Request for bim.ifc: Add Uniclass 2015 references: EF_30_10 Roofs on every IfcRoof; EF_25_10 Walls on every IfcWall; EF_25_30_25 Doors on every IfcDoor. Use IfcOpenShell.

First a look at what the model holds.

```python
import ifcopenshell

model = ifcopenshell.open("bim.ifc")
print(model.schema)
print("classifications:", [c.Name for c in model.by_type("IfcClassification")])
for ifc_class in ("IfcDoor", "IfcRoof", "IfcStair", "IfcWall", "IfcWindow"):
    print(ifc_class, len(model.by_type(ifc_class)))
```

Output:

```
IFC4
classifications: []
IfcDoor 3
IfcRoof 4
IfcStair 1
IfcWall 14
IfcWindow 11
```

```python
import ifcopenshell
import ifcopenshell.api.classification

model = ifcopenshell.open("bim.ifc")

system = ifcopenshell.api.classification.add_classification(model, classification="Uniclass 2015")

codes = {
    "IfcRoof": ("EF_30_10", "Roofs"),
    "IfcWall": ("EF_25_10", "Walls"),
    "IfcDoor": ("EF_25_30_25", "Doors"),
}
for ifc_class, (code, name) in codes.items():
    products = model.by_type(ifc_class)
    ifcopenshell.api.classification.add_reference(
        model, products=products, classification=system, identification=code, name=name
    )
    print(code, len(products))

model.write("bim_rev.ifc")
```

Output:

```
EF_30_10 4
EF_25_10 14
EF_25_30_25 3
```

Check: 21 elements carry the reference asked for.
